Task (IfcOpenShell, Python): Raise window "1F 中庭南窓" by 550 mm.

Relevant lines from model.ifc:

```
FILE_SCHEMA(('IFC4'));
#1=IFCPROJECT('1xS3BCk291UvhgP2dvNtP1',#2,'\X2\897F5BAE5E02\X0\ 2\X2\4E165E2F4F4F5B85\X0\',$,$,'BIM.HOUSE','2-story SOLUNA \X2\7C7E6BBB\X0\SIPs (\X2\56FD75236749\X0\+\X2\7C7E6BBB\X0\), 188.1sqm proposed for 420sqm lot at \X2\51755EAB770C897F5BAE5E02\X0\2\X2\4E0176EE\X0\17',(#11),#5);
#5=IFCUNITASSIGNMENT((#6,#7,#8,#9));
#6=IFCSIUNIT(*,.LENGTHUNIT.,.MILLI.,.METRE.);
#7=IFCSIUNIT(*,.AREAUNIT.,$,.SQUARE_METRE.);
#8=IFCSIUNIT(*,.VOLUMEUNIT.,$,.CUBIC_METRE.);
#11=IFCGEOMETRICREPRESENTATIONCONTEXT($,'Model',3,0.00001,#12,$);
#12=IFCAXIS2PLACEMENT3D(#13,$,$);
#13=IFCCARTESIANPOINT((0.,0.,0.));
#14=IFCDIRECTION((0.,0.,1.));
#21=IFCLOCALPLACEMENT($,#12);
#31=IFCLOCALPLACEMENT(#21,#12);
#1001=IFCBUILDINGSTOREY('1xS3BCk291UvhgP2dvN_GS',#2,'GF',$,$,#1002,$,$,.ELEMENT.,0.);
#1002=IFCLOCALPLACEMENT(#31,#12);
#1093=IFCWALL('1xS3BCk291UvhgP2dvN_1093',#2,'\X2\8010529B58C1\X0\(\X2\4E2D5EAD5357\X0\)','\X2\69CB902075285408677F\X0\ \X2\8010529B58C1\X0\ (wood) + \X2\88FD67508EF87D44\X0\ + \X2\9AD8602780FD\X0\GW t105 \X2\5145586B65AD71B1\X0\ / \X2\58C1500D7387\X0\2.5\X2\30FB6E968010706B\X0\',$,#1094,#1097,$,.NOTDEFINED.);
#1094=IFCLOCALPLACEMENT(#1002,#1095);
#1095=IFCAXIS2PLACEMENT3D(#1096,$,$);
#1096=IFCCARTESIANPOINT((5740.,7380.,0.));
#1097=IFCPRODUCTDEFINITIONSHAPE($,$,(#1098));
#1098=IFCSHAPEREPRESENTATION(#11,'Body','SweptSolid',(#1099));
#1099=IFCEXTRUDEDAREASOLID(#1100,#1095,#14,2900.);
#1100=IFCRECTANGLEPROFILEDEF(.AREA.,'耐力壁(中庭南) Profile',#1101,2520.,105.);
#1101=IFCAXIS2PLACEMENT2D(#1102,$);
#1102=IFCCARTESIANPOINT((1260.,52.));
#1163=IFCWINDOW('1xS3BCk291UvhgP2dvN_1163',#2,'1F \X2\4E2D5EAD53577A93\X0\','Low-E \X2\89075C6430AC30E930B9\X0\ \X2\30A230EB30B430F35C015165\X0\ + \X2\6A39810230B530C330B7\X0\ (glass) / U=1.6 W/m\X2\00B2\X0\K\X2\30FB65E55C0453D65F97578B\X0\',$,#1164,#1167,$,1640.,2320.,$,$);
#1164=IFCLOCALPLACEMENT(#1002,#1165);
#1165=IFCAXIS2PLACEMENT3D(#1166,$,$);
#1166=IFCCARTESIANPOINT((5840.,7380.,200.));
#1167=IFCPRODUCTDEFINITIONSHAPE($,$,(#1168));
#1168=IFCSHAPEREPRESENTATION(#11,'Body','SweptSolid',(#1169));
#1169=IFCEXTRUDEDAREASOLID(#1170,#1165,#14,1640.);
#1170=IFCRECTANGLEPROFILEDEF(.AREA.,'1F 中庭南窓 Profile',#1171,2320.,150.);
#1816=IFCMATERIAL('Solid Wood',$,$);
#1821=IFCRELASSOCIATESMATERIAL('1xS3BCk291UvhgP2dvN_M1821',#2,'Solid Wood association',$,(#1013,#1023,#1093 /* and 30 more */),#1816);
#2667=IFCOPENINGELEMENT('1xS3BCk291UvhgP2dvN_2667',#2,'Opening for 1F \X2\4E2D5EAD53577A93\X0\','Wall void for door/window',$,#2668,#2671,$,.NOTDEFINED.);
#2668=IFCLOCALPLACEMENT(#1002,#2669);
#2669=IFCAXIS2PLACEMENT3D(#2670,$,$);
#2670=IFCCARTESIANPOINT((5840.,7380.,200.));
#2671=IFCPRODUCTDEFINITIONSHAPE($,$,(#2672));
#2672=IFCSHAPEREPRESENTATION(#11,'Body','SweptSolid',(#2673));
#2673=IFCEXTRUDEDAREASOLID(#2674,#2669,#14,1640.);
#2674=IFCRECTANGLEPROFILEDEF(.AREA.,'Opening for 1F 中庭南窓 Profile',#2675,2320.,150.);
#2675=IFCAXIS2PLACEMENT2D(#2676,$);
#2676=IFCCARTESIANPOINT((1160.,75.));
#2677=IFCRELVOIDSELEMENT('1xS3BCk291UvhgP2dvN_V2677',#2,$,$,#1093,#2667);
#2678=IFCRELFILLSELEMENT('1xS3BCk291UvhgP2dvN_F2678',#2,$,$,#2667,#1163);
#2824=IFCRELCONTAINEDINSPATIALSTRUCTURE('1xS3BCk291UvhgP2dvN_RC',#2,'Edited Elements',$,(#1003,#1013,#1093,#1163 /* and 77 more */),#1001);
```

```python
import numpy as np
import ifcopenshell
import ifcopenshell.api.geometry
import ifcopenshell.util.placement
import ifcopenshell.util.unit

model = ifcopenshell.open("model.ifc")
unit_scale = ifcopenshell.util.unit.calculate_unit_scale(model)

window = model.by_id(1163)
opening = window.FillsVoids[0].RelatingOpeningElement
dz = 0.55 / unit_scale

shift = np.array([0.0, 0.0, dz])
# The window is not placed relative to its opening, so move both.
for product in (opening, window):
    matrix = ifcopenshell.util.placement.get_local_placement(product.ObjectPlacement)
    matrix[:3, 3] += shift
    ifcopenshell.api.geometry.edit_object_placement(model, product=product, matrix=matrix, is_si=False)

print(f"moved by {dz * unit_scale:+.3f} m")

model.write("model_updated.ifc")
```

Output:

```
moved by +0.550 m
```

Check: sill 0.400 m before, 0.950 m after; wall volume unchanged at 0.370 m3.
